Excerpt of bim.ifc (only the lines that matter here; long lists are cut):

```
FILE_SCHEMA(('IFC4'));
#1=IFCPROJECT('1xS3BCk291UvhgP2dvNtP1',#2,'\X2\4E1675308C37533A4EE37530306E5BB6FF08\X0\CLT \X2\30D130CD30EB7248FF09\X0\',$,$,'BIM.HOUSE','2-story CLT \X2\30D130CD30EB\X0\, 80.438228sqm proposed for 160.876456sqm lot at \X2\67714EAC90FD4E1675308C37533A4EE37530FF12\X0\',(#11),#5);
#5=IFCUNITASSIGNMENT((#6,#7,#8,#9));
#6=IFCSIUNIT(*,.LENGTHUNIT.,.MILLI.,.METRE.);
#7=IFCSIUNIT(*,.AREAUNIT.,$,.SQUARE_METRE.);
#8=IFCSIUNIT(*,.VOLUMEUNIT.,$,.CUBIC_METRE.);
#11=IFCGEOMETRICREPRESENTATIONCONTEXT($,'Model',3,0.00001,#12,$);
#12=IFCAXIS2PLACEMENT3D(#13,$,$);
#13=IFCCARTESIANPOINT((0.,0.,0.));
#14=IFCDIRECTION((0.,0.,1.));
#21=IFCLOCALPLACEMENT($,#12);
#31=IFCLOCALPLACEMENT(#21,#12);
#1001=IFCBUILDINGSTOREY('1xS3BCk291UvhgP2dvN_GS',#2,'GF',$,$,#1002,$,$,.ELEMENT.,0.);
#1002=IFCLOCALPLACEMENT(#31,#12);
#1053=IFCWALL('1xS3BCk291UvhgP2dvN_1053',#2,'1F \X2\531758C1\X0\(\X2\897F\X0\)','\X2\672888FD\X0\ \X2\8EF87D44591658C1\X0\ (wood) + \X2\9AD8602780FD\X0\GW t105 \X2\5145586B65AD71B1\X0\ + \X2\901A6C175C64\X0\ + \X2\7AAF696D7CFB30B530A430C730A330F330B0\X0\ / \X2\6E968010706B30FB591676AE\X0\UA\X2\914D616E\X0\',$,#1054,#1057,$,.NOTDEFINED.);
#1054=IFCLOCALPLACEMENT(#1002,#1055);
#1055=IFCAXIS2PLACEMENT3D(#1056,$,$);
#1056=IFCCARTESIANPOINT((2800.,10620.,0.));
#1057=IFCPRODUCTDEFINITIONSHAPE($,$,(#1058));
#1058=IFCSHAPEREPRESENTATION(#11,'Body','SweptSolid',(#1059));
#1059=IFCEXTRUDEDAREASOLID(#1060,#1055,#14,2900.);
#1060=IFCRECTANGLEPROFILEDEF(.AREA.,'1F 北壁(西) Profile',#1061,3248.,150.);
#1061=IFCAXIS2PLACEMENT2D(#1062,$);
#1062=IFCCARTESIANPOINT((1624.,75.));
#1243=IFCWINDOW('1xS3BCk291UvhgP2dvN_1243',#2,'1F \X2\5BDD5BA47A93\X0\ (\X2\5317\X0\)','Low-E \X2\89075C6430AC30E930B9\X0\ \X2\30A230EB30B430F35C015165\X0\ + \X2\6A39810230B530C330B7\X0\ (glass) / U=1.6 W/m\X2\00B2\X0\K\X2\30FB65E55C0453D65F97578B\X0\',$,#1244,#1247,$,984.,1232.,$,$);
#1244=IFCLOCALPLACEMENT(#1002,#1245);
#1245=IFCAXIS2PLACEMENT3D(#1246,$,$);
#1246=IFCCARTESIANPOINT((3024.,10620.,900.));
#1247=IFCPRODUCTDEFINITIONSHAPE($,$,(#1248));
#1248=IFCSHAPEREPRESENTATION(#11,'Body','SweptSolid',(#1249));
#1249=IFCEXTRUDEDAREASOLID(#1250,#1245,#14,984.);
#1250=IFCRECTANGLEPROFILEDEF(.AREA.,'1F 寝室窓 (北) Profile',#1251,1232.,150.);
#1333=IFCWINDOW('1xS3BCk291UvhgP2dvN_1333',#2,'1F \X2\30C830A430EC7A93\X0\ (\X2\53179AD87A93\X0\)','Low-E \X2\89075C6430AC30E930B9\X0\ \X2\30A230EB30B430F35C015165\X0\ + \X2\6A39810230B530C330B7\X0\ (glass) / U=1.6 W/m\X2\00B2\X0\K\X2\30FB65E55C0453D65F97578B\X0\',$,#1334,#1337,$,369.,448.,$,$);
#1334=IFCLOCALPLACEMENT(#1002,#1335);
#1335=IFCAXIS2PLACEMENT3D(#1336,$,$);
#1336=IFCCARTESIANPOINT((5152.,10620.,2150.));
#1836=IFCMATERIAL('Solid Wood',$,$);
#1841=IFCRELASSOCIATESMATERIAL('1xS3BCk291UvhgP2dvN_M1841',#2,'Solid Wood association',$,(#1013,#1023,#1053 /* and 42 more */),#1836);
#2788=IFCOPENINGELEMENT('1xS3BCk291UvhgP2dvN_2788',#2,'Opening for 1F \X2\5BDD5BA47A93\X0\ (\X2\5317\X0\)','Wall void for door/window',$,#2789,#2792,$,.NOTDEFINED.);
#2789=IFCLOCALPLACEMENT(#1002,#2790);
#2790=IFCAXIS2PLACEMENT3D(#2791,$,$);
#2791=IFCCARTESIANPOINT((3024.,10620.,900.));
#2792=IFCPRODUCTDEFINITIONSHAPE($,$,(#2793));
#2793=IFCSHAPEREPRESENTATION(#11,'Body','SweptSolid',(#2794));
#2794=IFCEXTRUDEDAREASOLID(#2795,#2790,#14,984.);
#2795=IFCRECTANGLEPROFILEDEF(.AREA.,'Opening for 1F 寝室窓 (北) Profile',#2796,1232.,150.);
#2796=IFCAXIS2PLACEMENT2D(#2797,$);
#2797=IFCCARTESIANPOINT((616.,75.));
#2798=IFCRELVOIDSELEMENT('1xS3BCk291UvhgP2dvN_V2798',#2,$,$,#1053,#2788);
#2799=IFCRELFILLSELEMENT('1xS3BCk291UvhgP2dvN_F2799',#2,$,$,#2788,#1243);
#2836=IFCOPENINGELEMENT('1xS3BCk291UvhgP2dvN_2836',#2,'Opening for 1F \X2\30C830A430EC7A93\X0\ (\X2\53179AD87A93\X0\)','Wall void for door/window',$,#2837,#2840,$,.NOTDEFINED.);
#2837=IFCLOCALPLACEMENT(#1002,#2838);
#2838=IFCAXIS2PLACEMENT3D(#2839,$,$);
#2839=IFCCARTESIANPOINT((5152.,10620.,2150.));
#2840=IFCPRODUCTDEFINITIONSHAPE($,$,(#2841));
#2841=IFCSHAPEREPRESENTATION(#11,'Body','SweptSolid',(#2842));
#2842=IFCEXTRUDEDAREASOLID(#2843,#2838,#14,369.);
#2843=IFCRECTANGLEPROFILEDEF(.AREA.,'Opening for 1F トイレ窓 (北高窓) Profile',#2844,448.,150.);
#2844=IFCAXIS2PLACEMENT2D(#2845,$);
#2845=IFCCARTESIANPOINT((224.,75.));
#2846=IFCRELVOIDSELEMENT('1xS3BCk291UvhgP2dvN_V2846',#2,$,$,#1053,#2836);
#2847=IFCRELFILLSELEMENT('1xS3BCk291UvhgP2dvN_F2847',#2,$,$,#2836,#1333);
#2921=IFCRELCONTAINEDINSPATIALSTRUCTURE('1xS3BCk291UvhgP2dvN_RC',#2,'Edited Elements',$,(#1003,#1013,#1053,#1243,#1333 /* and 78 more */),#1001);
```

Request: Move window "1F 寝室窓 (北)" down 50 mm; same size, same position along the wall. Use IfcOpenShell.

```python
import numpy as np
import ifcopenshell
import ifcopenshell.api.geometry
import ifcopenshell.util.placement
import ifcopenshell.util.unit

model = ifcopenshell.open("bim.ifc")
unit_scale = ifcopenshell.util.unit.calculate_unit_scale(model)

window = model.by_id(1243)
opening = window.FillsVoids[0].RelatingOpeningElement
dz = -50.0

shift = np.array([0.0, 0.0, dz])
# The window is not placed relative to its opening, so move both.
for product in (opening, window):
    matrix = ifcopenshell.util.placement.get_local_placement(product.ObjectPlacement)
    matrix[:3, 3] += shift
    ifcopenshell.api.geometry.edit_object_placement(model, product=product, matrix=matrix, is_si=False)

print(f"moved by {dz * unit_scale:+.3f} m")

model.write("bim_rev.ifc")
```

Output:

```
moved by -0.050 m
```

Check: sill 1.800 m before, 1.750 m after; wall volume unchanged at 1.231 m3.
